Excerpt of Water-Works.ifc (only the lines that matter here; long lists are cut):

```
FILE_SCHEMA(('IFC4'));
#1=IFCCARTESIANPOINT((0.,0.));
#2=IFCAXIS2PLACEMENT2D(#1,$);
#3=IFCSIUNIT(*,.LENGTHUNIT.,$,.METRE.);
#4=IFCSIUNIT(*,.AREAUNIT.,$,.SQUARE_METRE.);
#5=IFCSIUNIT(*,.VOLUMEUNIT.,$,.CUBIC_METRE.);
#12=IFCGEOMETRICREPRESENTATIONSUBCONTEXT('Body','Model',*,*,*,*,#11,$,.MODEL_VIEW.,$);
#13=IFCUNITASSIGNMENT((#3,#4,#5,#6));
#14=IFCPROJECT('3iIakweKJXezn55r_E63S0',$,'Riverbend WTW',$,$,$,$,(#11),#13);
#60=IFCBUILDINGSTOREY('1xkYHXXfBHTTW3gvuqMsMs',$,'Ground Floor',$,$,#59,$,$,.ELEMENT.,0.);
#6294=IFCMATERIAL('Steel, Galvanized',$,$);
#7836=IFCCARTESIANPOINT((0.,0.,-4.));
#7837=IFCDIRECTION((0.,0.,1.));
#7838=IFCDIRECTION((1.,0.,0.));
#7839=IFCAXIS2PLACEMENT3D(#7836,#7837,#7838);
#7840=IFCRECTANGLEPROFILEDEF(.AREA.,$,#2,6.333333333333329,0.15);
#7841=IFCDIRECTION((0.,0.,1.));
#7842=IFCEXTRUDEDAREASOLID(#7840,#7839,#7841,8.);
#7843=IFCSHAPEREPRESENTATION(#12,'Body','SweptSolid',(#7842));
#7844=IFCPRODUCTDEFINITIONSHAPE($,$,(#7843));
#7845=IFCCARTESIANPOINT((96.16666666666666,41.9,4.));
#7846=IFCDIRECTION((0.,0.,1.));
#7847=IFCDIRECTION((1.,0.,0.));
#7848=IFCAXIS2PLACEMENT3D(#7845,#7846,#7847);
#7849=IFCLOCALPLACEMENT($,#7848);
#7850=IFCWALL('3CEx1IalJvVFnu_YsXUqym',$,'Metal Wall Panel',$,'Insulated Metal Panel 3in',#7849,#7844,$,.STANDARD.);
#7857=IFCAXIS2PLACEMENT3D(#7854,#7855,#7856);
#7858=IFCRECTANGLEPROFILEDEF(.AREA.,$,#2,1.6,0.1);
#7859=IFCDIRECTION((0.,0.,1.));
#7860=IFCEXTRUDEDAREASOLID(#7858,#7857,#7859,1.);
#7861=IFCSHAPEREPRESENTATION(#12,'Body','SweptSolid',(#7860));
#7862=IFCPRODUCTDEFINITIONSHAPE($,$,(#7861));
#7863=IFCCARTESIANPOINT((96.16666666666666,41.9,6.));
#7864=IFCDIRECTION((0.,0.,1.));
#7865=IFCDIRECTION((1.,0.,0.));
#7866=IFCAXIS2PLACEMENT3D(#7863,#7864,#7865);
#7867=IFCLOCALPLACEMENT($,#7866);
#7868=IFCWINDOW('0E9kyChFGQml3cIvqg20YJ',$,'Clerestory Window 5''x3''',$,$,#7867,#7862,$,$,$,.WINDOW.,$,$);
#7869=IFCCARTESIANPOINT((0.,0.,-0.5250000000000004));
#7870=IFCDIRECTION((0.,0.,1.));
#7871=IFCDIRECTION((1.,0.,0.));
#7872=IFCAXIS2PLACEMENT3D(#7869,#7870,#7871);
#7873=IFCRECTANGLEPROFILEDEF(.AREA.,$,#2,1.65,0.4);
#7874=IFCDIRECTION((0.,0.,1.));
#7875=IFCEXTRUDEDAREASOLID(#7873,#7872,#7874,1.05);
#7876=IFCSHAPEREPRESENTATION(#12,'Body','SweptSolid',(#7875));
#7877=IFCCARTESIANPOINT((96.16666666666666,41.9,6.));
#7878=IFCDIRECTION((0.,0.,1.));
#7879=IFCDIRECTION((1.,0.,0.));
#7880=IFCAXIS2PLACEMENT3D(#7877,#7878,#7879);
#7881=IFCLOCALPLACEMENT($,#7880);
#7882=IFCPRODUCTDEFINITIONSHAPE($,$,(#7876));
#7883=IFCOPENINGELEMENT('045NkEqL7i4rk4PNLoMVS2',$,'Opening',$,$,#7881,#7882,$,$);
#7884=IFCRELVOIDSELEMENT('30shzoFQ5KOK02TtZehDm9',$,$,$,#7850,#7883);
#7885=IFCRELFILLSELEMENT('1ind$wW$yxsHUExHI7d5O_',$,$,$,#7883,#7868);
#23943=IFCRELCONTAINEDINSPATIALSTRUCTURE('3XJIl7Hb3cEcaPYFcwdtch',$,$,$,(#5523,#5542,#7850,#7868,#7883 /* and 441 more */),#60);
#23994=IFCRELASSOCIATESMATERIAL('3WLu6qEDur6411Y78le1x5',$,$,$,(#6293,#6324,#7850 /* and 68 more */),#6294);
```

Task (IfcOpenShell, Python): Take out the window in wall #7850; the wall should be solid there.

```python
import ifcopenshell
import ifcopenshell.api.feature
import ifcopenshell.api.root
import ifcopenshell.geom
import ifcopenshell.util.shape

model = ifcopenshell.open("Water-Works.ifc")
settings = ifcopenshell.geom.settings()


def volume(element):
    """Net volume in cubic metres, openings subtracted."""
    shape = ifcopenshell.geom.create_shape(settings, element)
    return ifcopenshell.util.shape.get_volume(shape.geometry)


window = model.by_id(7868)
opening = window.FillsVoids[0].RelatingOpeningElement
wall = opening.VoidsElements[0].RelatingBuildingElement
before = volume(wall)

ifcopenshell.api.root.remove_product(model, product=window)
ifcopenshell.api.feature.remove_feature(model, feature=opening)

after = volume(wall)

print(f"wall volume {before:.3f} -> {after:.3f} m3")

model.write("Water-Works-out.ifc")
```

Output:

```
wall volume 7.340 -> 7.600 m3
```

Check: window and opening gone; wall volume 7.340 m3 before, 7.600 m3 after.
